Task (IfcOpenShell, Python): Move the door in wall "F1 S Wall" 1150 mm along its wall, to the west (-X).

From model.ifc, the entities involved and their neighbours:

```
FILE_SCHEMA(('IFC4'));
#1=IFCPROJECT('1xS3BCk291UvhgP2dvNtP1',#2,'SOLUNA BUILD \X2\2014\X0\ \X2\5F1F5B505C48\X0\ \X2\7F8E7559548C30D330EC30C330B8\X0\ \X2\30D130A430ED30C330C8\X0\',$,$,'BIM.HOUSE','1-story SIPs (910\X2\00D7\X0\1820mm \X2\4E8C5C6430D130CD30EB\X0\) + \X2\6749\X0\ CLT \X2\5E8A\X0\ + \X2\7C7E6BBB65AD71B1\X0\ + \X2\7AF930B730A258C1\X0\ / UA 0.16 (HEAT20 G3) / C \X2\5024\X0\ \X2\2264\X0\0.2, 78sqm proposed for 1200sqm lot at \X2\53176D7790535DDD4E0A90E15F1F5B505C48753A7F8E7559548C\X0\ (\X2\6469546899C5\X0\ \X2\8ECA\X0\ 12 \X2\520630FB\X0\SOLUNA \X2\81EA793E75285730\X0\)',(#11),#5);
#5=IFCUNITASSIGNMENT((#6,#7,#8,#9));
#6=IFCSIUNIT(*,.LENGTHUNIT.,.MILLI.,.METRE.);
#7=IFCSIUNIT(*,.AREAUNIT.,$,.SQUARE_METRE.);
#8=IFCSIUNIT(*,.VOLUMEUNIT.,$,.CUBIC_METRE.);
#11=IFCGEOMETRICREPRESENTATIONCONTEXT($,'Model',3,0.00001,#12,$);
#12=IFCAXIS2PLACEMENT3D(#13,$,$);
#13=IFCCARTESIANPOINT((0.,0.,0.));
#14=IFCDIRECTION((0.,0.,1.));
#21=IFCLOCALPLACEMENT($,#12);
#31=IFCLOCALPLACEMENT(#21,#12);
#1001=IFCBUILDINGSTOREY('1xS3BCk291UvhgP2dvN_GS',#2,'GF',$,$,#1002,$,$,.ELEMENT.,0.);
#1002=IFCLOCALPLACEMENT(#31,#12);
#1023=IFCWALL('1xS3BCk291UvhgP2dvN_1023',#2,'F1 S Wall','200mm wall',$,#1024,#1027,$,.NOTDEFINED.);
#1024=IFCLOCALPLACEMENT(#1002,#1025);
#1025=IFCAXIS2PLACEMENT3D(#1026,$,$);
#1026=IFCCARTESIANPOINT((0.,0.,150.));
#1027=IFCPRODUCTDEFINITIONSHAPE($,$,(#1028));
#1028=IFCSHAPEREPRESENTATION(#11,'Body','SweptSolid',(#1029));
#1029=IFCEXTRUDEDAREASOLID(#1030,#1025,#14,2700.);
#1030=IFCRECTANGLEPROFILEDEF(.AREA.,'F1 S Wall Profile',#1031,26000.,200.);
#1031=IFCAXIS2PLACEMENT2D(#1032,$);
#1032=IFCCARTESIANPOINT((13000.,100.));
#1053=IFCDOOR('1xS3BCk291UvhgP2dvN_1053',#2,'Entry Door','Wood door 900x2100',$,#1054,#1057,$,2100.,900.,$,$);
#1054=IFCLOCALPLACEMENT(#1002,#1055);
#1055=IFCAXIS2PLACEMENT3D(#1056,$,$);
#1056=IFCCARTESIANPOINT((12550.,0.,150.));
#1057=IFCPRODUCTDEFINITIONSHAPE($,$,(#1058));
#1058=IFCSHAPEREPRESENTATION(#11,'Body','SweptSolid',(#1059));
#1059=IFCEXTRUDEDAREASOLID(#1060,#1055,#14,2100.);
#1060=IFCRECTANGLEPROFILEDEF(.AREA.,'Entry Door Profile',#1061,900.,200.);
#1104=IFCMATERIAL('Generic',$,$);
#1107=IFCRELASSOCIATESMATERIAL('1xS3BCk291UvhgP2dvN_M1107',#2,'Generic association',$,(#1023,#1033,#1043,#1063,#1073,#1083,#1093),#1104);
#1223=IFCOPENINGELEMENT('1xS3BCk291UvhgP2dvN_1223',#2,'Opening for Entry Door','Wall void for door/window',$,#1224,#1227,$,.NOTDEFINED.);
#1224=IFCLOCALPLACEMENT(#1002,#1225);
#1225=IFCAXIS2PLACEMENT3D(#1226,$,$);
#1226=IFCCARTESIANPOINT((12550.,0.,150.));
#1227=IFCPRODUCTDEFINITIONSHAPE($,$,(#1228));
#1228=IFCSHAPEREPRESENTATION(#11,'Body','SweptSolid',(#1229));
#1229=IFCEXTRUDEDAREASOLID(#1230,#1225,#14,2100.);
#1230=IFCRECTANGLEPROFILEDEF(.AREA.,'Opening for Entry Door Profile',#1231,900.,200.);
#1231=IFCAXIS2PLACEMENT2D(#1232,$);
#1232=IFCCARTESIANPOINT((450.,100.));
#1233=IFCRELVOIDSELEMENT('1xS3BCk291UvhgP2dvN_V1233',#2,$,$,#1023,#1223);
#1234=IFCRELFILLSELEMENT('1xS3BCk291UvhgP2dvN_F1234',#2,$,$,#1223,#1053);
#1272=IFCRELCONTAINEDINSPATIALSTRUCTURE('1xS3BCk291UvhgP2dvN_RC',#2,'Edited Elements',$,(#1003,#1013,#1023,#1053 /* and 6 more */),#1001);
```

```python
import ifcopenshell
import ifcopenshell.api.geometry
import ifcopenshell.util.placement

model = ifcopenshell.open("model.ifc")

door = model.by_guid("1xS3BCk291UvhgP2dvN_1053")
opening = door.FillsVoids[0].RelatingOpeningElement
wall = opening.VoidsElements[0].RelatingBuildingElement

wall_matrix = ifcopenshell.util.placement.get_local_placement(wall.ObjectPlacement)
shift = wall_matrix[:3, 0] * -1150.0
before = ifcopenshell.util.placement.get_local_placement(door.ObjectPlacement)[:3, 3].copy()

# The door is not placed relative to its opening, so move both.
for product in (opening, door):
    matrix = ifcopenshell.util.placement.get_local_placement(product.ObjectPlacement)
    matrix[:3, 3] += shift
    ifcopenshell.api.geometry.edit_object_placement(model, product=product, matrix=matrix, is_si=False)

after = ifcopenshell.util.placement.get_local_placement(door.ObjectPlacement)[:3, 3]
print("door moved by", (after - before).round(3) + 0.0)

model.write("model-out.ifc")
```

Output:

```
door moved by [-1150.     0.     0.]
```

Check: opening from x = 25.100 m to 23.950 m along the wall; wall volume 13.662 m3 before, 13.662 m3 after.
